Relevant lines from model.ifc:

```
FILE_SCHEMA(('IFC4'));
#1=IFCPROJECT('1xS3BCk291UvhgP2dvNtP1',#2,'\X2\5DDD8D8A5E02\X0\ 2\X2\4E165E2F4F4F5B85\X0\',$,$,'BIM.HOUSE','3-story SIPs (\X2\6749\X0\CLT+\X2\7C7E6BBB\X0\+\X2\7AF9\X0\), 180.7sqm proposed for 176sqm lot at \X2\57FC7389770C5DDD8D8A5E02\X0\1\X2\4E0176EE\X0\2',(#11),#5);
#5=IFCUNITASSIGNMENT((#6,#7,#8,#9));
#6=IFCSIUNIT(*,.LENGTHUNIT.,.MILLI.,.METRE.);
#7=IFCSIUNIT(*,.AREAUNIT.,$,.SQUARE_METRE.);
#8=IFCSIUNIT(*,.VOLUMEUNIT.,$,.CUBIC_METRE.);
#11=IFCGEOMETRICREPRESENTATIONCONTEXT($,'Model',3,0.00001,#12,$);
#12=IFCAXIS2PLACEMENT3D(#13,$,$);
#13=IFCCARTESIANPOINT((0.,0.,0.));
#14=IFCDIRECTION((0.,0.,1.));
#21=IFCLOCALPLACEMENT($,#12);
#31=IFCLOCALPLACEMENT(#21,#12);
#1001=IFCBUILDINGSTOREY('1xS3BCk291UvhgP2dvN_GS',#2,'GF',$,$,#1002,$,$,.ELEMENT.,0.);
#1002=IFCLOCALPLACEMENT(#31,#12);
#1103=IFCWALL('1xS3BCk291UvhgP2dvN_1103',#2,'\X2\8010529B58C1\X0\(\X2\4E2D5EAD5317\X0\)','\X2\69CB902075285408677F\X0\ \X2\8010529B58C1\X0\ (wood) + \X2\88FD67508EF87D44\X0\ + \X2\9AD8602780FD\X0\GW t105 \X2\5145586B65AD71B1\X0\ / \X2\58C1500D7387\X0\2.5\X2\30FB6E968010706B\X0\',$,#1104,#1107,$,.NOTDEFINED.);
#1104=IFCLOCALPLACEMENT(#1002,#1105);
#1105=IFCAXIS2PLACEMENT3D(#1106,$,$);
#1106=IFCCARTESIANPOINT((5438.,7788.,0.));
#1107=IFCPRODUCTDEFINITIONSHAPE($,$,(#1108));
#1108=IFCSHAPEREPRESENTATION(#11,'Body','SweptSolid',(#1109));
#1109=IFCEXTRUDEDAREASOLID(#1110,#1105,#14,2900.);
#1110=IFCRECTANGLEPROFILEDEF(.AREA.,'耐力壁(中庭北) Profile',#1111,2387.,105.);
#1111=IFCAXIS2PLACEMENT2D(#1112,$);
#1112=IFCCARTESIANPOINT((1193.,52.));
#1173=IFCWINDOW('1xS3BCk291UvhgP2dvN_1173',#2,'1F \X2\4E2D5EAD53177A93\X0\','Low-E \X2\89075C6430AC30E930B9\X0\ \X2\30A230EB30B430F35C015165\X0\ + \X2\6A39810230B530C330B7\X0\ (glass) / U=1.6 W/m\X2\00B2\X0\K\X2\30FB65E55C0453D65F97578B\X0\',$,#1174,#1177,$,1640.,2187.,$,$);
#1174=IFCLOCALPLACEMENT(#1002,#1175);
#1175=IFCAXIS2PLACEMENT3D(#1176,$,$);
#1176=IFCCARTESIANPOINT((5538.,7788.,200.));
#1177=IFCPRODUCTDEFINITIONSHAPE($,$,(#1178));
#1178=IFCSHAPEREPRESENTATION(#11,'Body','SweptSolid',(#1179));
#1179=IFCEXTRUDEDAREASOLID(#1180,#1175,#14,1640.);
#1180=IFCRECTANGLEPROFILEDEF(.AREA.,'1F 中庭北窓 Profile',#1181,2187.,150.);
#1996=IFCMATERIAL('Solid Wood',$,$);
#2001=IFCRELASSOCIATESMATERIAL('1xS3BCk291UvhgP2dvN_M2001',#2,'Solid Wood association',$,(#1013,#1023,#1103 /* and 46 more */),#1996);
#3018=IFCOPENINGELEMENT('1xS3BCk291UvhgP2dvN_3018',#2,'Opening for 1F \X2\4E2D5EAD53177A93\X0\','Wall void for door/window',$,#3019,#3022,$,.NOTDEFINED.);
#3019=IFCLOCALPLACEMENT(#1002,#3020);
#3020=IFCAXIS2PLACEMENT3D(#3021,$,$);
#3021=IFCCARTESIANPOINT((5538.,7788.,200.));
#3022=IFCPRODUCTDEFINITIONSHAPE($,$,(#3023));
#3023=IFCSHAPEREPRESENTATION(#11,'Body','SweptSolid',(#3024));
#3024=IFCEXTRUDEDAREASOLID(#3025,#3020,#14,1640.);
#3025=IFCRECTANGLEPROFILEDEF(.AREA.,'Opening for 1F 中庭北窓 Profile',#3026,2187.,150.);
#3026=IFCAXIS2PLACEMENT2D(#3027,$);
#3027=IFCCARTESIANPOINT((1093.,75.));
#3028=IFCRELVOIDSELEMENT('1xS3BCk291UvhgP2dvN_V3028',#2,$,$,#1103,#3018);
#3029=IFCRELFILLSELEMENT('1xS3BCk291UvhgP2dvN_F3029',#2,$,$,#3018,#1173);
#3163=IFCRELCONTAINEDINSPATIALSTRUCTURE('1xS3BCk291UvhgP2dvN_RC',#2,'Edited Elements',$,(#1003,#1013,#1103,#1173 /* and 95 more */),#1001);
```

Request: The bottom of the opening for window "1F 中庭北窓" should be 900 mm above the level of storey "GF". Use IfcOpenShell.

```python
import numpy as np
import ifcopenshell
import ifcopenshell.api.geometry
import ifcopenshell.geom
import ifcopenshell.util.element
import ifcopenshell.util.placement
import ifcopenshell.util.shape
import ifcopenshell.util.unit

model = ifcopenshell.open("model.ifc")
unit_scale = ifcopenshell.util.unit.calculate_unit_scale(model)

window = model.by_guid("1xS3BCk291UvhgP2dvN_1173")
opening = window.FillsVoids[0].RelatingOpeningElement
storey = ifcopenshell.util.element.get_container(window, ifc_class="IfcBuildingStorey")
level = ifcopenshell.util.placement.get_local_placement(storey.ObjectPlacement)[2, 3]

# The opening's origin need not be at the sill, so measure its lowest point.
shape = ifcopenshell.geom.create_shape(ifcopenshell.geom.settings(), opening)
bottom = ifcopenshell.util.shape.get_shape_bottom_elevation(shape, shape.geometry) / unit_scale
dz = level + 900.0 - bottom

shift = np.array([0.0, 0.0, dz])
# The window is not placed relative to its opening, so move both.
for product in (opening, window):
    matrix = ifcopenshell.util.placement.get_local_placement(product.ObjectPlacement)
    matrix[:3, 3] += shift
    ifcopenshell.api.geometry.edit_object_placement(model, product=product, matrix=matrix, is_si=False)

print(f"moved by {dz * unit_scale:+.3f} m")

model.write("model-out.ifc")
```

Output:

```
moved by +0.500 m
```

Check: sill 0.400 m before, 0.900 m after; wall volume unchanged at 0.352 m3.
